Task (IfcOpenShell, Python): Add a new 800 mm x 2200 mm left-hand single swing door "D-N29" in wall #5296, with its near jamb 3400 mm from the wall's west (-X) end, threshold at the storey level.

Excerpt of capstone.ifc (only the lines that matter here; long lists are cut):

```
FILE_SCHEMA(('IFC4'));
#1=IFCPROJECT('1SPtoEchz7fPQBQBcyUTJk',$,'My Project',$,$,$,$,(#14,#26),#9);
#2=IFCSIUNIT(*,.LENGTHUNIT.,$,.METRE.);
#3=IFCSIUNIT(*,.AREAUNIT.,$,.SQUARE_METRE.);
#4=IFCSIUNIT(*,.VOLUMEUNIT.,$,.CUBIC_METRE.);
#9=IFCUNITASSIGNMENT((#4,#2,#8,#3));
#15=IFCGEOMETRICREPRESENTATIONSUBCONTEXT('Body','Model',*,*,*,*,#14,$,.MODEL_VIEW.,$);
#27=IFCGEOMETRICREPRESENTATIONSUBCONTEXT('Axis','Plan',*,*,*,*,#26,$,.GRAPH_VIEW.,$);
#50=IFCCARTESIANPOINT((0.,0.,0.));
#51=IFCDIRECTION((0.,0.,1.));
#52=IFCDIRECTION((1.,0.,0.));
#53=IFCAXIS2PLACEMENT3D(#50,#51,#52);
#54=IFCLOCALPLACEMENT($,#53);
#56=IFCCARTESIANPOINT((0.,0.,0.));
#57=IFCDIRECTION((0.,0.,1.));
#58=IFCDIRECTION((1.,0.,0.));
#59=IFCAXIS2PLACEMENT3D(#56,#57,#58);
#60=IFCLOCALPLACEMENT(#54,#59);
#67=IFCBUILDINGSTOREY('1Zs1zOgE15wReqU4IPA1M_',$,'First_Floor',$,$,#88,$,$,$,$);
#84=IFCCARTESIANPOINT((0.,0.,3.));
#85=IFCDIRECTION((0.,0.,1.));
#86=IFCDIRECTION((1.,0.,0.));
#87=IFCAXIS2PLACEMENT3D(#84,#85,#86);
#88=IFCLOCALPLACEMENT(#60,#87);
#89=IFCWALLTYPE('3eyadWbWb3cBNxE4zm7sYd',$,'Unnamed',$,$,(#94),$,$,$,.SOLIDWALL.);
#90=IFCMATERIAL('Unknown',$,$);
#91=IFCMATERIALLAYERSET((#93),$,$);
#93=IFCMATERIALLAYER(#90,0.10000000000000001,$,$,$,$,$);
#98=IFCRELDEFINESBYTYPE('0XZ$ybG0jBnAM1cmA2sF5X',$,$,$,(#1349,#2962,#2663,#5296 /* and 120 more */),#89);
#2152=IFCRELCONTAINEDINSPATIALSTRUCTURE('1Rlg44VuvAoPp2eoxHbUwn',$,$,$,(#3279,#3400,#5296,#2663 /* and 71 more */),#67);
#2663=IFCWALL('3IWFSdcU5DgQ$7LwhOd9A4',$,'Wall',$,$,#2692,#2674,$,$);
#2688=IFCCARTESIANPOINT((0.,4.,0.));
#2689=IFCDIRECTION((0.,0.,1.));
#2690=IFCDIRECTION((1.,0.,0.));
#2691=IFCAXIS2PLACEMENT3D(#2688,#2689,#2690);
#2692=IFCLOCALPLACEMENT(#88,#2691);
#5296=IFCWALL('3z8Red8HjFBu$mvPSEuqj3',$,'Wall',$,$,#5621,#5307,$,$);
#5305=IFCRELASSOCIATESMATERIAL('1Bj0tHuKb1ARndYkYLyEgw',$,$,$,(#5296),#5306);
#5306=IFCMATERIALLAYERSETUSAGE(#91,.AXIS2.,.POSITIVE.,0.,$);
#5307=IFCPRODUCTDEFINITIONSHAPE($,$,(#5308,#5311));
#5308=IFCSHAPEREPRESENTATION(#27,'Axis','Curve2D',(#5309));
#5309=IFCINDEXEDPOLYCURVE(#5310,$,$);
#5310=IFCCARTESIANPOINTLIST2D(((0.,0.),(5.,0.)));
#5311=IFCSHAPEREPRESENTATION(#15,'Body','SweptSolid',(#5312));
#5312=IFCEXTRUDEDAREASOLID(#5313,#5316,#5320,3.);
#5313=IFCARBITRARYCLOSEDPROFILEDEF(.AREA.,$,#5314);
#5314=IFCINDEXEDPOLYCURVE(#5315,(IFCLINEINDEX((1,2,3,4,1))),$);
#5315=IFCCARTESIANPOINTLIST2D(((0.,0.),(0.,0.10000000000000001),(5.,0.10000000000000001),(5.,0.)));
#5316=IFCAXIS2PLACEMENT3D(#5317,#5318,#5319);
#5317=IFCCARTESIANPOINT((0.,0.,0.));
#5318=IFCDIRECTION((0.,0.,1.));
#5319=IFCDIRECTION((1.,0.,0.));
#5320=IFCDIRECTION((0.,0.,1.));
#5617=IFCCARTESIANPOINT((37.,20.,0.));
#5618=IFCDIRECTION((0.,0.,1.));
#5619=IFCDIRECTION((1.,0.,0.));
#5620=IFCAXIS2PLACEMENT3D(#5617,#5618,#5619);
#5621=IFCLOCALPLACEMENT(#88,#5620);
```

```python
import numpy as np
import ifcopenshell
import ifcopenshell.api.feature
import ifcopenshell.api.geometry
import ifcopenshell.api.root
import ifcopenshell.api.spatial
import ifcopenshell.geom
import ifcopenshell.util.element
import ifcopenshell.util.placement
import ifcopenshell.util.representation
import ifcopenshell.util.shape
import ifcopenshell.util.unit

model = ifcopenshell.open("capstone.ifc")
unit_scale = ifcopenshell.util.unit.calculate_unit_scale(model)
settings = ifcopenshell.geom.settings()


def volume(element):
    """Net volume in cubic metres, openings subtracted."""
    shape = ifcopenshell.geom.create_shape(settings, element)
    return ifcopenshell.util.shape.get_volume(shape.geometry)


wall = model.by_guid("3z8Red8HjFBu$mvPSEuqj3")
storey = ifcopenshell.util.element.get_container(wall, ifc_class="IfcBuildingStorey")
context = ifcopenshell.util.representation.get_context(model, "Model", "Body", "MODEL_VIEW")
before = volume(wall)

width, height, from_end, sill = 0.8, 2.2, 3.4, 0.0  # metres

# The wall runs along its own X axis, and the end named is its -X end.
wall_shape = ifcopenshell.geom.create_shape(settings, wall)
x, y, z = ifcopenshell.util.shape.get_vertices(wall_shape.geometry).T
start = x.min() + from_end
face, thickness = float(y.min()), float(y.max() - y.min())
wall_matrix = ifcopenshell.util.placement.get_local_placement(wall.ObjectPlacement)
level = ifcopenshell.util.placement.get_local_placement(storey.ObjectPlacement)[2, 3]


def in_wall(x, y):
    """Placement at x, y metres in the wall's axes, at sill height."""
    matrix = wall_matrix.copy()
    matrix[:, 3] = wall_matrix @ np.array([x / unit_scale, y / unit_scale, 0.0, 1.0])
    matrix[2, 3] = level + sill / unit_scale
    return matrix


# Opening: a box that overshoots both wall faces by 50 mm.
opening = ifcopenshell.api.root.create_entity(model, ifc_class="IfcOpeningElement", predefined_type="OPENING")
box = ifcopenshell.api.geometry.add_wall_representation(
    model, context=context, length=width, height=height, thickness=thickness + 0.1
)
ifcopenshell.api.geometry.assign_representation(model, product=opening, representation=box)
ifcopenshell.api.geometry.edit_object_placement(model, product=opening, matrix=in_wall(start, face - 0.05), is_si=False)
ifcopenshell.api.feature.add_feature(model, feature=opening, element=wall)

door = ifcopenshell.api.root.create_entity(model, ifc_class="IfcDoor", name="D-N29", predefined_type="DOOR")
door.OverallWidth, door.OverallHeight = width / unit_scale, height / unit_scale
door.OperationType = "SINGLE_SWING_LEFT"
body = ifcopenshell.api.geometry.add_door_representation(
    model,
    context=context,
    overall_width=door.OverallWidth,
    overall_height=door.OverallHeight,
    operation_type="SINGLE_SWING_LEFT",
    lining_properties={"LiningDepth": thickness / unit_scale, "ThresholdDepth": thickness / unit_scale},
)
ifcopenshell.api.geometry.assign_representation(model, product=door, representation=body)
ifcopenshell.api.spatial.assign_container(model, products=[door], relating_structure=storey)
ifcopenshell.api.feature.add_filling(model, opening=opening, element=door)

# The lining spans the wall, so the door starts at the wall face.
ifcopenshell.api.geometry.edit_object_placement(model, product=door, matrix=in_wall(start, face), is_si=False)

after = volume(wall)

print(f"wall volume {before:.3f} -> {after:.3f} m3")

model.write("capstone_edited.ifc")
```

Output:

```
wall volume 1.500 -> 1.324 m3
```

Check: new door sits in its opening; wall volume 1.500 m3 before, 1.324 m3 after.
